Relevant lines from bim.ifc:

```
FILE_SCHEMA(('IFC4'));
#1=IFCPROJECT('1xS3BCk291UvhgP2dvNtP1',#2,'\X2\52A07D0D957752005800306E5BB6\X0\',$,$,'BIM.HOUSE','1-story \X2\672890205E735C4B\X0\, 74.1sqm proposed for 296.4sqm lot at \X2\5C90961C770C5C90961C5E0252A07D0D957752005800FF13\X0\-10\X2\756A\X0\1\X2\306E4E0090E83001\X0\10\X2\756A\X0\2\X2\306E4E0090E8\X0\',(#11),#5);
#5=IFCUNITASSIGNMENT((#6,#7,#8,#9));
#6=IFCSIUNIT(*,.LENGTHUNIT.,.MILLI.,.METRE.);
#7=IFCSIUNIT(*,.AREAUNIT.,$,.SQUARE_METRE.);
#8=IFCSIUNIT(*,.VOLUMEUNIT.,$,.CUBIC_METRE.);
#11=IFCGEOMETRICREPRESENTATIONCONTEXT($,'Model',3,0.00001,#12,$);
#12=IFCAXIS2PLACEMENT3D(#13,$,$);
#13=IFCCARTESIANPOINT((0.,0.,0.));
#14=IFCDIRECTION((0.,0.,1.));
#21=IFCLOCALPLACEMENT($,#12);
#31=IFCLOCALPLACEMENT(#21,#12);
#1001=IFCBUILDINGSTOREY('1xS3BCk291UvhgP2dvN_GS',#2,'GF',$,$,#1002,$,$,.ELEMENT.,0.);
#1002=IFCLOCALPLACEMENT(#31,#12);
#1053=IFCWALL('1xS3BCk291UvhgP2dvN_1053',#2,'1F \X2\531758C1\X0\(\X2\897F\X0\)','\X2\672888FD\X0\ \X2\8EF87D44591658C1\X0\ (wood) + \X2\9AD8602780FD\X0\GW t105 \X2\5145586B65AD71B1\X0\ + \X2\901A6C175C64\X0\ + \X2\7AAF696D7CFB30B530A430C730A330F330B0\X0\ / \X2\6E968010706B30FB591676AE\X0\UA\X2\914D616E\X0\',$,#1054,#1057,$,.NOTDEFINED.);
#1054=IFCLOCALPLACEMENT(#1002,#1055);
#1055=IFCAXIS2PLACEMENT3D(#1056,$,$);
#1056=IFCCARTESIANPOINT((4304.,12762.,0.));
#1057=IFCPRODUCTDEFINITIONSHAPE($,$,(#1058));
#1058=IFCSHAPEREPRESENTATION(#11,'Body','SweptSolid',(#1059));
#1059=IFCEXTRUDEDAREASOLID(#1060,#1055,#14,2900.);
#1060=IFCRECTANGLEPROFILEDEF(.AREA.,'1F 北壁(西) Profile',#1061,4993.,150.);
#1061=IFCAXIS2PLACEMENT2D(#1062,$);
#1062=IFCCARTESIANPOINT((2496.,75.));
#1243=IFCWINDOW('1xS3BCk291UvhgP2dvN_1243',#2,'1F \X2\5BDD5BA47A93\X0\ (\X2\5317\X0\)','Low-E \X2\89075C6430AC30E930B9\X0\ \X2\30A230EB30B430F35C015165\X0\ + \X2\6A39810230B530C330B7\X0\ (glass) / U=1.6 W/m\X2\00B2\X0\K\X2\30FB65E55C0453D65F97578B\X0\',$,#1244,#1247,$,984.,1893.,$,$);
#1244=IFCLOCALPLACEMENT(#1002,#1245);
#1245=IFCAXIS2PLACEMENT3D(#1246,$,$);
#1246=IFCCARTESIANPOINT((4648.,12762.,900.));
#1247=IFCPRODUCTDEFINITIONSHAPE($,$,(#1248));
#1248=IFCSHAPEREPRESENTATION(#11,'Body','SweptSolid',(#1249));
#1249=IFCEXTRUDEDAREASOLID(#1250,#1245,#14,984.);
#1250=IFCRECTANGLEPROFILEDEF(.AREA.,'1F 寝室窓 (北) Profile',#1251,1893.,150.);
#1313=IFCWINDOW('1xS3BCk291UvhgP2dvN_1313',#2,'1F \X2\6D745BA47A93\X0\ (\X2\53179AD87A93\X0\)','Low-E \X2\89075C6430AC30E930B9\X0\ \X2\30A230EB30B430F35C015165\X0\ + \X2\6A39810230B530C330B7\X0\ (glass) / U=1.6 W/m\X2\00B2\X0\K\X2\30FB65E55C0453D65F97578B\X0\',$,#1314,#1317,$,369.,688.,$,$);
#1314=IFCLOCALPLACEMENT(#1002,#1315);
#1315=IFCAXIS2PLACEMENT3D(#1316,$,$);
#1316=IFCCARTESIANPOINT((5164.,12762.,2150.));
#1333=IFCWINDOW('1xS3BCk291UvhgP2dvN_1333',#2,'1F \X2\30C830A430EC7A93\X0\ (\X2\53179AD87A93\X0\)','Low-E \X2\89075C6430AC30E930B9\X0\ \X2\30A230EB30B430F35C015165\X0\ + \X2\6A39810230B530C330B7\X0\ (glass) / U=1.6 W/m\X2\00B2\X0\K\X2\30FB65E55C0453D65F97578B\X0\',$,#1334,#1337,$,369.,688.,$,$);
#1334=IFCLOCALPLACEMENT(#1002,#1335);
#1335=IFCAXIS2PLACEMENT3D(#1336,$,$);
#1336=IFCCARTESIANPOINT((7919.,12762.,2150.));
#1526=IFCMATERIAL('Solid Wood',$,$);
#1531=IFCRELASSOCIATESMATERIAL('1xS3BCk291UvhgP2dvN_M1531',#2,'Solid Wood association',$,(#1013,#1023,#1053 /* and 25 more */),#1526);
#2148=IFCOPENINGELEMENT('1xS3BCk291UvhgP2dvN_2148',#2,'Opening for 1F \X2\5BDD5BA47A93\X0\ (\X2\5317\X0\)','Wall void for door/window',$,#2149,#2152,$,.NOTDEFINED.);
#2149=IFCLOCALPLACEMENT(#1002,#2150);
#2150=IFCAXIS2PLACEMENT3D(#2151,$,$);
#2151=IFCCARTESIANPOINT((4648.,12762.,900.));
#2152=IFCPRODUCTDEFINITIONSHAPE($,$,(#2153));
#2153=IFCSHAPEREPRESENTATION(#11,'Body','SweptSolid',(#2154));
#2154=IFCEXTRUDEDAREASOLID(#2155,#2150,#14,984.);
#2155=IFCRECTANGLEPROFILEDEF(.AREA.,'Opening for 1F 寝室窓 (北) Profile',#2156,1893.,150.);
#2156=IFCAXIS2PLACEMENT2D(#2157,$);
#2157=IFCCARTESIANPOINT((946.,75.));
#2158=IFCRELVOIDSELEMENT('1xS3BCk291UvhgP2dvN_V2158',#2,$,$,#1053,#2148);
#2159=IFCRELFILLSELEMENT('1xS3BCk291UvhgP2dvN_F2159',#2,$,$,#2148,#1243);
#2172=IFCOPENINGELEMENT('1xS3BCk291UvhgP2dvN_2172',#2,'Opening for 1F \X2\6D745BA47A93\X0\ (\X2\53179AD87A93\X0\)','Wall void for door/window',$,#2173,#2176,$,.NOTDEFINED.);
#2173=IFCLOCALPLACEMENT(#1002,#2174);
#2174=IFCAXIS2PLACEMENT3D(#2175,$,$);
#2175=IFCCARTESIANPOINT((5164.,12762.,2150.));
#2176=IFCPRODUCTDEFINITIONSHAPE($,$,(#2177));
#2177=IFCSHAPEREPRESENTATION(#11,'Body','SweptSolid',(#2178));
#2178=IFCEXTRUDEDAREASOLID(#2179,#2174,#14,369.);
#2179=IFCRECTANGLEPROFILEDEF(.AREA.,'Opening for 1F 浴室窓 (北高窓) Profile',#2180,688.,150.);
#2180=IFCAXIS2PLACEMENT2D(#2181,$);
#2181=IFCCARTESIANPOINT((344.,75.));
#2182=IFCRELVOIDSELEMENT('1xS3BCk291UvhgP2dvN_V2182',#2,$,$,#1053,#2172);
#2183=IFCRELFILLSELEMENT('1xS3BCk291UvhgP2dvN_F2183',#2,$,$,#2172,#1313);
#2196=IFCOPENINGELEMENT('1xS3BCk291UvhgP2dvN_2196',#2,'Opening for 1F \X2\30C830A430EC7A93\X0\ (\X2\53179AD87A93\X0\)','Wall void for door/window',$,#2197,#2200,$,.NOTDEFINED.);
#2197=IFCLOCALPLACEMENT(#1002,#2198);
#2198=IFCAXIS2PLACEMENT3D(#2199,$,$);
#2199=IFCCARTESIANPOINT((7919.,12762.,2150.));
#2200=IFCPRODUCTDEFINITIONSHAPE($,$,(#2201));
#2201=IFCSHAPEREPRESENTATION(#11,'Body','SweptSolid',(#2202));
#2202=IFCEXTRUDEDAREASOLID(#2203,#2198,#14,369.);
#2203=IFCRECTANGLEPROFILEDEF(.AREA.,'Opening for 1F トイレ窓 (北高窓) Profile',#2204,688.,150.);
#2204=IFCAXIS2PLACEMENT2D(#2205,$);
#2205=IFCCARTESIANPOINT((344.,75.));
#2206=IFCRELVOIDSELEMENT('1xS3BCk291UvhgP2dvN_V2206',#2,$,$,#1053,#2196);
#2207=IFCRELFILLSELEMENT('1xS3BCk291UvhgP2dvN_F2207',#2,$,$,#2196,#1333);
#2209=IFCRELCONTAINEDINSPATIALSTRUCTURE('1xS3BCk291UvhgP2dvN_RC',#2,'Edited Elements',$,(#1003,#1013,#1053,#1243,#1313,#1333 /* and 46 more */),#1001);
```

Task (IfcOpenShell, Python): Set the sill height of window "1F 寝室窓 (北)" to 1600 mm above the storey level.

```python
import numpy as np
import ifcopenshell
import ifcopenshell.api.geometry
import ifcopenshell.geom
import ifcopenshell.util.element
import ifcopenshell.util.placement
import ifcopenshell.util.shape
import ifcopenshell.util.unit

model = ifcopenshell.open("bim.ifc")
unit_scale = ifcopenshell.util.unit.calculate_unit_scale(model)

window = model.by_guid("1xS3BCk291UvhgP2dvN_1243")
opening = window.FillsVoids[0].RelatingOpeningElement
storey = ifcopenshell.util.element.get_container(window, ifc_class="IfcBuildingStorey")
level = ifcopenshell.util.placement.get_local_placement(storey.ObjectPlacement)[2, 3]

# The opening's origin need not be at the sill, so measure its lowest point.
shape = ifcopenshell.geom.create_shape(ifcopenshell.geom.settings(), opening)
bottom = ifcopenshell.util.shape.get_shape_bottom_elevation(shape, shape.geometry) / unit_scale
dz = level + 1.6 / unit_scale - bottom

shift = np.array([0.0, 0.0, dz])
# The window is not placed relative to its opening, so move both.
for product in (opening, window):
    matrix = ifcopenshell.util.placement.get_local_placement(product.ObjectPlacement)
    matrix[:3, 3] += shift
    ifcopenshell.api.geometry.edit_object_placement(model, product=product, matrix=matrix, is_si=False)

print(f"moved by {dz * unit_scale:+.3f} m")

model.write("bim_v2.ifc")
```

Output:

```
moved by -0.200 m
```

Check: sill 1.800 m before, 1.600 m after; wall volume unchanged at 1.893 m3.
